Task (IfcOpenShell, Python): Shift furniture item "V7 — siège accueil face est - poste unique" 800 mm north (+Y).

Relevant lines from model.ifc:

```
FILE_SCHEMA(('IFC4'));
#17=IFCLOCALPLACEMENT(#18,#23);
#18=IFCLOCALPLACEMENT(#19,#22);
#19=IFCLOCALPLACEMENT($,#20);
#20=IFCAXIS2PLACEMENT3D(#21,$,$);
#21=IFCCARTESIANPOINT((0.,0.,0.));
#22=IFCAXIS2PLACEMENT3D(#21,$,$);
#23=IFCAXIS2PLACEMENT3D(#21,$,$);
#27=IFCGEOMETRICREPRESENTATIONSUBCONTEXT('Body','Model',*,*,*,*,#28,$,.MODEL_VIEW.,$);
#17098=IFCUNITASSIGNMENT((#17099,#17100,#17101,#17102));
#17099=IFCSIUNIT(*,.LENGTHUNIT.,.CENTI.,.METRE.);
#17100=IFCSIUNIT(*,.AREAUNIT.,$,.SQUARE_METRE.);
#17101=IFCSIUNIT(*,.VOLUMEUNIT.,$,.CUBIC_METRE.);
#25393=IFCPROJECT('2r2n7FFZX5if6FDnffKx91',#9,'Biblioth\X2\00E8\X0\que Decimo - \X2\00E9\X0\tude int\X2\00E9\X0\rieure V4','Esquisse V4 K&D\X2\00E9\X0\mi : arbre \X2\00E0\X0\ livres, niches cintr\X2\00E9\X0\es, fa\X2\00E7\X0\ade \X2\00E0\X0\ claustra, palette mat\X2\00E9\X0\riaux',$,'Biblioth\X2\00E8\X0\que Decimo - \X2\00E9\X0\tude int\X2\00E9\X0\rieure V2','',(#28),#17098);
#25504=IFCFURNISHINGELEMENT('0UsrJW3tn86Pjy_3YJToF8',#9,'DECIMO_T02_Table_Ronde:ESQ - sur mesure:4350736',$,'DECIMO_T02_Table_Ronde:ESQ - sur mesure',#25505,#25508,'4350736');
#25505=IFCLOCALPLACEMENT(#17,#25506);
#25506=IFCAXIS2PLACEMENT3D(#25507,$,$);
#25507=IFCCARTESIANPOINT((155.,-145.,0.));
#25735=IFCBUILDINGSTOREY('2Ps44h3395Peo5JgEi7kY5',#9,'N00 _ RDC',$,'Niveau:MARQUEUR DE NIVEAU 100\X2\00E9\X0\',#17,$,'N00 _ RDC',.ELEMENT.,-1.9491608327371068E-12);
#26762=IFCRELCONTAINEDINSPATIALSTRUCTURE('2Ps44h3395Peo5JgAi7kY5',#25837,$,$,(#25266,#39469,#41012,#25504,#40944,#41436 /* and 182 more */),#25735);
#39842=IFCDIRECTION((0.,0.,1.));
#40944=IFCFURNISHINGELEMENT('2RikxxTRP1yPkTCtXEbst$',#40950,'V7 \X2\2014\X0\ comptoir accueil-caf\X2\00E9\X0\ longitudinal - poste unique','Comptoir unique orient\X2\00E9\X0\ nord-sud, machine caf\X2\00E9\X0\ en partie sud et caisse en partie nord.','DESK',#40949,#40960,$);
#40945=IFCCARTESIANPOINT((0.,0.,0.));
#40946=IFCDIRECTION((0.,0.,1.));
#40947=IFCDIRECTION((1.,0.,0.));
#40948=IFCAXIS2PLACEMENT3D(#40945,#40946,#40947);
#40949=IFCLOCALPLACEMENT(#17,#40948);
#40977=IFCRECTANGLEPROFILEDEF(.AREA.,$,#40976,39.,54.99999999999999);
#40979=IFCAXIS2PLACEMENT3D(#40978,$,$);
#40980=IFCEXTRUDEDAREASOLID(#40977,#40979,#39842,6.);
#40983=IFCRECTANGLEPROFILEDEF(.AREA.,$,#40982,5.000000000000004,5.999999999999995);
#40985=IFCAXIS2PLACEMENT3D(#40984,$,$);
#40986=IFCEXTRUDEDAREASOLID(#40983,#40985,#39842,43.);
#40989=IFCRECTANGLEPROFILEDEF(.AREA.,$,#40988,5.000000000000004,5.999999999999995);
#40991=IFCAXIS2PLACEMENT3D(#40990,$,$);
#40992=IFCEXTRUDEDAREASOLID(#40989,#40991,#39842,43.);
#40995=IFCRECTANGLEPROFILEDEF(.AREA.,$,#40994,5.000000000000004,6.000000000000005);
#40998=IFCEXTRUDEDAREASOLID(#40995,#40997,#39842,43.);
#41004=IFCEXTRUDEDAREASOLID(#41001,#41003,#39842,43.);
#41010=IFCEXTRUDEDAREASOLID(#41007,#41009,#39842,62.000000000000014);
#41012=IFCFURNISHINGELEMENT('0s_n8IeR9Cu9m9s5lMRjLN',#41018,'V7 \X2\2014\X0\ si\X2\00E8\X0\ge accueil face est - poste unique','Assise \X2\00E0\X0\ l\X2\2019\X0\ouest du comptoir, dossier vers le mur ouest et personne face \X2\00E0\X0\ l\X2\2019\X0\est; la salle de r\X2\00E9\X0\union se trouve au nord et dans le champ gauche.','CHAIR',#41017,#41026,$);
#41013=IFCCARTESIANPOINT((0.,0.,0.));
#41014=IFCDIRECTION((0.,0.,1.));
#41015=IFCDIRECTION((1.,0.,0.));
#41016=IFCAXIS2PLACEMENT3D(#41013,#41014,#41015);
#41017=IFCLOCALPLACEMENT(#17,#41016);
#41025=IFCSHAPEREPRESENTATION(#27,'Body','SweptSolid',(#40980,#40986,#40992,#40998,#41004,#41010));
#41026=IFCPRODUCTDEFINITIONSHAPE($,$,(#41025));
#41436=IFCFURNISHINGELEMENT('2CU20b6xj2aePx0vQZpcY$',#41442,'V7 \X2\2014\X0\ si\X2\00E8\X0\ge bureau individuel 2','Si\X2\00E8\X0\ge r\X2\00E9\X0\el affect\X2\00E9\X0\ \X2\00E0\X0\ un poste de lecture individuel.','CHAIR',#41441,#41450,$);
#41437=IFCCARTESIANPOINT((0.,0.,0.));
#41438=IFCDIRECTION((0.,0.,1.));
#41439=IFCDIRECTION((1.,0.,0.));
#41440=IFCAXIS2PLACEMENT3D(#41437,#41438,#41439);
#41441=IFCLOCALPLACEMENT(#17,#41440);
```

```python
import ifcopenshell
import ifcopenshell.api.geometry
import ifcopenshell.util.placement
import ifcopenshell.util.unit

model = ifcopenshell.open("model.ifc")
unit_scale = ifcopenshell.util.unit.calculate_unit_scale(model)

item = model.by_guid("0s_n8IeR9Cu9m9s5lMRjLN")
matrix = ifcopenshell.util.placement.get_local_placement(item.ObjectPlacement)
matrix[1, 3] += 0.8 / unit_scale
ifcopenshell.api.geometry.edit_object_placement(model, product=item, matrix=matrix, is_si=False)

print(ifcopenshell.util.placement.get_local_placement(item.ObjectPlacement).round(3) + 0.0)

model.write("model_rev.ifc")
```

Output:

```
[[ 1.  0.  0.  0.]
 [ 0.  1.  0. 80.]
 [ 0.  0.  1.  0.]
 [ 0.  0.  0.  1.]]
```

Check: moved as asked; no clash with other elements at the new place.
